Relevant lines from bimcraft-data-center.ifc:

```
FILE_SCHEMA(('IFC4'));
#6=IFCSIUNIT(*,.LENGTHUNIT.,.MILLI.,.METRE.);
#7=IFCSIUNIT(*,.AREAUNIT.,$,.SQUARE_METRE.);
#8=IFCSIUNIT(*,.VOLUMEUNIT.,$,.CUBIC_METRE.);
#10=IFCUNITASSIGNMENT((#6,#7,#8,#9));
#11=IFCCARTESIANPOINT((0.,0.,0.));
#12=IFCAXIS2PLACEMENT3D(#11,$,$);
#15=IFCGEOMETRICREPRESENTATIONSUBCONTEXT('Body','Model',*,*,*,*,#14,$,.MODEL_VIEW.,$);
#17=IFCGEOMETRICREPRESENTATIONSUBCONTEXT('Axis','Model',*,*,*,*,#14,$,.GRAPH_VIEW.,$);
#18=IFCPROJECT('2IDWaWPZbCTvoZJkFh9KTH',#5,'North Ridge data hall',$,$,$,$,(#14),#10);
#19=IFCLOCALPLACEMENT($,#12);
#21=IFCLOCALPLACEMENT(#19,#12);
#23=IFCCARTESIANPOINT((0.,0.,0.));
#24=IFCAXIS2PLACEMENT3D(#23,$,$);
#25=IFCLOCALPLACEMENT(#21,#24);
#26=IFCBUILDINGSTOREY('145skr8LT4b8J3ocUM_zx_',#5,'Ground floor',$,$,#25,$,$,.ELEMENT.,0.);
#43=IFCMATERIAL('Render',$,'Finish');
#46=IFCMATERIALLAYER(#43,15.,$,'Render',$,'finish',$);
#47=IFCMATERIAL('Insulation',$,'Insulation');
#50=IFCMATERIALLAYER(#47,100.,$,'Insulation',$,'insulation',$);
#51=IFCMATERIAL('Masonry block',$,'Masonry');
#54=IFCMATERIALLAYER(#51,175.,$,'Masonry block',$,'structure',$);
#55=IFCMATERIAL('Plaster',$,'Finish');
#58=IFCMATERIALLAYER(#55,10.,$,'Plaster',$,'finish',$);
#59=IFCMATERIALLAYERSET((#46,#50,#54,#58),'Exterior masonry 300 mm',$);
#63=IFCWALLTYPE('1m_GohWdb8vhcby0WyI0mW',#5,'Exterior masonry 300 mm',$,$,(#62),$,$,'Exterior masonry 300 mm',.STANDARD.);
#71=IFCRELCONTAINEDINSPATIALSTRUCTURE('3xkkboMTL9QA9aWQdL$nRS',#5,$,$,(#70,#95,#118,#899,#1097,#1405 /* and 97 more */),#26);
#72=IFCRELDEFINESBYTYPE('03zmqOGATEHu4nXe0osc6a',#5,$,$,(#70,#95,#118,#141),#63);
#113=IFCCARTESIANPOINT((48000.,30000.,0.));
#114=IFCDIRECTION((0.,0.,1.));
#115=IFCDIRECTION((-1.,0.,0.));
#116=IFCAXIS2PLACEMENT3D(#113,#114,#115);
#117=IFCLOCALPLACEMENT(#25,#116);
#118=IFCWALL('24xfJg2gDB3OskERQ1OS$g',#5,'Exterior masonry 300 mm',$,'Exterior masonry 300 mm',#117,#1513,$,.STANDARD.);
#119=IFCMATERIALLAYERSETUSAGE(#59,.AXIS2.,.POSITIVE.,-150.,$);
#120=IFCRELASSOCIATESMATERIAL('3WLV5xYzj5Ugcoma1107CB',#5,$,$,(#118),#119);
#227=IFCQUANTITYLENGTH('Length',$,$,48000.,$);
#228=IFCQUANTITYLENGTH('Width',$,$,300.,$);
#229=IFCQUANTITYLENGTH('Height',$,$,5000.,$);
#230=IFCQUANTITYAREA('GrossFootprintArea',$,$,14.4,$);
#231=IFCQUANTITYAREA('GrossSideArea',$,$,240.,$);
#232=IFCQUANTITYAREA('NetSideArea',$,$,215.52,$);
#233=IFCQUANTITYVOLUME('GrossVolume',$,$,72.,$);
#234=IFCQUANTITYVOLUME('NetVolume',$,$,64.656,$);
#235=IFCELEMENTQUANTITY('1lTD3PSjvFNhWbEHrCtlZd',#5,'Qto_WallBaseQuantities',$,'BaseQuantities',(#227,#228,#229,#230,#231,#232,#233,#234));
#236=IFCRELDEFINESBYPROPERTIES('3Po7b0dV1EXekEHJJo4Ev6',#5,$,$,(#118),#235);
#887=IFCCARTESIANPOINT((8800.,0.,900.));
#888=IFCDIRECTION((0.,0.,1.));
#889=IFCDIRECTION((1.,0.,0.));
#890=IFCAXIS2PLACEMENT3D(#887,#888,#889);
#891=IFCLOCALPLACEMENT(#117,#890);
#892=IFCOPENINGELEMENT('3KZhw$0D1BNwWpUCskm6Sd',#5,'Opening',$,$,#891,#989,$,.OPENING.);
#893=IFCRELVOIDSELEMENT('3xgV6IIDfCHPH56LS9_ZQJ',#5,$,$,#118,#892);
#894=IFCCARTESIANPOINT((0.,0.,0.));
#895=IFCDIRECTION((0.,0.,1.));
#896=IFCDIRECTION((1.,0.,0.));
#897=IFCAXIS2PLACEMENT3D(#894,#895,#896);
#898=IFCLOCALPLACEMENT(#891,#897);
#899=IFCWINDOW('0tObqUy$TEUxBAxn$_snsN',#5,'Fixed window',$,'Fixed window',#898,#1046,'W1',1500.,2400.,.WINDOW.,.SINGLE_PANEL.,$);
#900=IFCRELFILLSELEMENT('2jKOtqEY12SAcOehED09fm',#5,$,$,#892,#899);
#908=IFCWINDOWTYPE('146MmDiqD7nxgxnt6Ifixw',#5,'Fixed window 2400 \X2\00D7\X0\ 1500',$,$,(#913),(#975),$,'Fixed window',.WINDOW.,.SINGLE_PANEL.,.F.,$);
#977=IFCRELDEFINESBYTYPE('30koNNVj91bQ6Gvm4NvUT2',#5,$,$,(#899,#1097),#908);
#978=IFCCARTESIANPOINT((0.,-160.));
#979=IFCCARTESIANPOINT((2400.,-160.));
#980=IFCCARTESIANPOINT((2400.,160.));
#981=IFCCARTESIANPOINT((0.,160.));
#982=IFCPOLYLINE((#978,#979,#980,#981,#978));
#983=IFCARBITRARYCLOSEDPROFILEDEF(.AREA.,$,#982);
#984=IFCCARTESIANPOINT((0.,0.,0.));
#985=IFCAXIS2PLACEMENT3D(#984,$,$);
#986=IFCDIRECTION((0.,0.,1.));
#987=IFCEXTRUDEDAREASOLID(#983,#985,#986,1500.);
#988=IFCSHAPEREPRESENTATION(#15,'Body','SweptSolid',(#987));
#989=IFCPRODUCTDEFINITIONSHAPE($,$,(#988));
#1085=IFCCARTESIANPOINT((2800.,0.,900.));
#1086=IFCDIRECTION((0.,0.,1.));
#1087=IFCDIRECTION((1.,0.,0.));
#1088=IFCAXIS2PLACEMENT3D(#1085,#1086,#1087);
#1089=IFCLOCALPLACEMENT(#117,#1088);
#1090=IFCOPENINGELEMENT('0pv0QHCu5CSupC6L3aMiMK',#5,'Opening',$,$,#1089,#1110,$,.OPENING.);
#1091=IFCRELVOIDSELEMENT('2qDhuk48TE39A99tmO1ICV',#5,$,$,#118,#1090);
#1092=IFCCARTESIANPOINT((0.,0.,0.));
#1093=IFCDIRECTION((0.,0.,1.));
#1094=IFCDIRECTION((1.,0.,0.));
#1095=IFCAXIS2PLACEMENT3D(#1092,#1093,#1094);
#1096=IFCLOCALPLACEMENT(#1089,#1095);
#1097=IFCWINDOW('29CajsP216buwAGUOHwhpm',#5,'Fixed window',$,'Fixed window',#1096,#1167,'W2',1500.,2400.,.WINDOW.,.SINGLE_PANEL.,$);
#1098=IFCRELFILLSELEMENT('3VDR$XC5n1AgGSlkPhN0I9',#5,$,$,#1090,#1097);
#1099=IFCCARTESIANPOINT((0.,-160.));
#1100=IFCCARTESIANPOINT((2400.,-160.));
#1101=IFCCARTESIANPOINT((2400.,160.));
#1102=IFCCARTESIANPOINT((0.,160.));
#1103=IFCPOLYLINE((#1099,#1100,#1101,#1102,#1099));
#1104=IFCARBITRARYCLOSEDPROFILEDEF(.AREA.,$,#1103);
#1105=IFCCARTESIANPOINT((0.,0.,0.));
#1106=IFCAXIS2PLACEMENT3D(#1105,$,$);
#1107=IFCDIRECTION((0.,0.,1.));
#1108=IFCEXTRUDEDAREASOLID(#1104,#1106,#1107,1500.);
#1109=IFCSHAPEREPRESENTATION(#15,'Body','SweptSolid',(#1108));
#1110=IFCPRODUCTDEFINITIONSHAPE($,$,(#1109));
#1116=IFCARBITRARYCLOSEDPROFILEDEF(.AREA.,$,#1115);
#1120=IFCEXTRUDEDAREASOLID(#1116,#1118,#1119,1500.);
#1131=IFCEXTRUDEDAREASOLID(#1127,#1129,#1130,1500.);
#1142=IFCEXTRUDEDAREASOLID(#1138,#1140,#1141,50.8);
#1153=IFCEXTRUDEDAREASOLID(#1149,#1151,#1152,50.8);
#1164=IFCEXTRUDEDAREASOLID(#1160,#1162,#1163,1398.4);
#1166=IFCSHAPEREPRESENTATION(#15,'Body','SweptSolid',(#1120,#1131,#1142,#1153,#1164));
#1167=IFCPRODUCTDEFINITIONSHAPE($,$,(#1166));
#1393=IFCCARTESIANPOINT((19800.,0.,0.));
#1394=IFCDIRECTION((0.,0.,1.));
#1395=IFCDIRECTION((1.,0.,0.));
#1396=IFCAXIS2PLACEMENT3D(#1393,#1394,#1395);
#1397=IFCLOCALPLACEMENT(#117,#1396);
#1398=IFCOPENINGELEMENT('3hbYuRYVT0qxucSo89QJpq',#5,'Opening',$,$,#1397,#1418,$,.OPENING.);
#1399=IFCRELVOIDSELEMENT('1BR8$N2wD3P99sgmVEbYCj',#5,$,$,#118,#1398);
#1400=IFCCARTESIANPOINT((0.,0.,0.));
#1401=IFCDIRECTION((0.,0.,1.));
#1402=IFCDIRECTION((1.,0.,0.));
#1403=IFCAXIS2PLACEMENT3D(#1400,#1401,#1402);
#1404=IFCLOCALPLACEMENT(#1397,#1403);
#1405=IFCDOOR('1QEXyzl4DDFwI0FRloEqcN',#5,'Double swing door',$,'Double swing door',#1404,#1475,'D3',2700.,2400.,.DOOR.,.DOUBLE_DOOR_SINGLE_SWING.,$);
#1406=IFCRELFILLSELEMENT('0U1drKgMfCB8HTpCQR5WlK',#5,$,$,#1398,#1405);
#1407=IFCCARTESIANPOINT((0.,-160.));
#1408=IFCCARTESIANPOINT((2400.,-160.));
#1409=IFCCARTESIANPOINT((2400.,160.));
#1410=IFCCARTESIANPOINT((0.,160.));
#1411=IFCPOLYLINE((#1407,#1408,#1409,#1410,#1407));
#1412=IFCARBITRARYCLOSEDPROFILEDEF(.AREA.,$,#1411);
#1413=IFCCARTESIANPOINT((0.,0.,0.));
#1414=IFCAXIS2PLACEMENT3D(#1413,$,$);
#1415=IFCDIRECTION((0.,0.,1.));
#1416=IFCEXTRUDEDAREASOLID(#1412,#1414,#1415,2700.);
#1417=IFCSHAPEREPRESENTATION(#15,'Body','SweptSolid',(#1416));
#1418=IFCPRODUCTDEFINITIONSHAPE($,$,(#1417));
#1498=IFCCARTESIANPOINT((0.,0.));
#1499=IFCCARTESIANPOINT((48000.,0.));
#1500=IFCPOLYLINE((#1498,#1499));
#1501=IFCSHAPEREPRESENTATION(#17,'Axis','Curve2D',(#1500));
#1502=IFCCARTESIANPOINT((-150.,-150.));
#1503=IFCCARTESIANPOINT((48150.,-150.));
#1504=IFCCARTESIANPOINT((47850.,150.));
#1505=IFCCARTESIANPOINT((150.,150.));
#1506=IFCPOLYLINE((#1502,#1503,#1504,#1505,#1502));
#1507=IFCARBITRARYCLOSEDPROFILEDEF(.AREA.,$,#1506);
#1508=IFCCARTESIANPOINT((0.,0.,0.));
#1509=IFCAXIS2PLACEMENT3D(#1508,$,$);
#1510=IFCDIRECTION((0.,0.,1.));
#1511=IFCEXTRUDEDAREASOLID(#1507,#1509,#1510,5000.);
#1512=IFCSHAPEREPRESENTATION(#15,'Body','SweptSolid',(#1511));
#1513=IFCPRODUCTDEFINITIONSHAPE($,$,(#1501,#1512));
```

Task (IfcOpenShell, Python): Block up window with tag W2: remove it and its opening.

```python
import ifcopenshell
import ifcopenshell.api.feature
import ifcopenshell.api.pset
import ifcopenshell.api.root
import ifcopenshell.geom
import ifcopenshell.util.element
import ifcopenshell.util.shape
import ifcopenshell.util.unit

model = ifcopenshell.open("bimcraft-data-center.ifc")
area_scale = ifcopenshell.util.unit.calculate_unit_scale(model, "AREAUNIT")
volume_scale = ifcopenshell.util.unit.calculate_unit_scale(model, "VOLUMEUNIT")
settings = ifcopenshell.geom.settings()


def volume(element):
    """Net volume in cubic metres, openings subtracted."""
    shape = ifcopenshell.geom.create_shape(settings, element)
    return ifcopenshell.util.shape.get_volume(shape.geometry)


window = model.by_id(1097)
opening = window.FillsVoids[0].RelatingOpeningElement
wall = opening.VoidsElements[0].RelatingBuildingElement
before = volume(wall)

ifcopenshell.api.root.remove_product(model, product=window)
ifcopenshell.api.feature.remove_feature(model, feature=opening)

after = volume(wall)
thickness = 0.3  # wall thickness in metres

# Update the wall's stored quantities.
qto = model.by_id(ifcopenshell.util.element.get_pset(wall, "Qto_WallBaseQuantities", should_inherit=False)["id"])
ifcopenshell.api.pset.edit_qto(model, qto=qto, properties={
    "NetSideArea": after / thickness / area_scale,
    "NetVolume": after / volume_scale,
})

print(f"wall volume {before:.3f} -> {after:.3f} m3")

model.write("bimcraft-data-center_v2.ifc")
```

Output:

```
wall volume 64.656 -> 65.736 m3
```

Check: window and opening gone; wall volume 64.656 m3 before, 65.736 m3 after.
